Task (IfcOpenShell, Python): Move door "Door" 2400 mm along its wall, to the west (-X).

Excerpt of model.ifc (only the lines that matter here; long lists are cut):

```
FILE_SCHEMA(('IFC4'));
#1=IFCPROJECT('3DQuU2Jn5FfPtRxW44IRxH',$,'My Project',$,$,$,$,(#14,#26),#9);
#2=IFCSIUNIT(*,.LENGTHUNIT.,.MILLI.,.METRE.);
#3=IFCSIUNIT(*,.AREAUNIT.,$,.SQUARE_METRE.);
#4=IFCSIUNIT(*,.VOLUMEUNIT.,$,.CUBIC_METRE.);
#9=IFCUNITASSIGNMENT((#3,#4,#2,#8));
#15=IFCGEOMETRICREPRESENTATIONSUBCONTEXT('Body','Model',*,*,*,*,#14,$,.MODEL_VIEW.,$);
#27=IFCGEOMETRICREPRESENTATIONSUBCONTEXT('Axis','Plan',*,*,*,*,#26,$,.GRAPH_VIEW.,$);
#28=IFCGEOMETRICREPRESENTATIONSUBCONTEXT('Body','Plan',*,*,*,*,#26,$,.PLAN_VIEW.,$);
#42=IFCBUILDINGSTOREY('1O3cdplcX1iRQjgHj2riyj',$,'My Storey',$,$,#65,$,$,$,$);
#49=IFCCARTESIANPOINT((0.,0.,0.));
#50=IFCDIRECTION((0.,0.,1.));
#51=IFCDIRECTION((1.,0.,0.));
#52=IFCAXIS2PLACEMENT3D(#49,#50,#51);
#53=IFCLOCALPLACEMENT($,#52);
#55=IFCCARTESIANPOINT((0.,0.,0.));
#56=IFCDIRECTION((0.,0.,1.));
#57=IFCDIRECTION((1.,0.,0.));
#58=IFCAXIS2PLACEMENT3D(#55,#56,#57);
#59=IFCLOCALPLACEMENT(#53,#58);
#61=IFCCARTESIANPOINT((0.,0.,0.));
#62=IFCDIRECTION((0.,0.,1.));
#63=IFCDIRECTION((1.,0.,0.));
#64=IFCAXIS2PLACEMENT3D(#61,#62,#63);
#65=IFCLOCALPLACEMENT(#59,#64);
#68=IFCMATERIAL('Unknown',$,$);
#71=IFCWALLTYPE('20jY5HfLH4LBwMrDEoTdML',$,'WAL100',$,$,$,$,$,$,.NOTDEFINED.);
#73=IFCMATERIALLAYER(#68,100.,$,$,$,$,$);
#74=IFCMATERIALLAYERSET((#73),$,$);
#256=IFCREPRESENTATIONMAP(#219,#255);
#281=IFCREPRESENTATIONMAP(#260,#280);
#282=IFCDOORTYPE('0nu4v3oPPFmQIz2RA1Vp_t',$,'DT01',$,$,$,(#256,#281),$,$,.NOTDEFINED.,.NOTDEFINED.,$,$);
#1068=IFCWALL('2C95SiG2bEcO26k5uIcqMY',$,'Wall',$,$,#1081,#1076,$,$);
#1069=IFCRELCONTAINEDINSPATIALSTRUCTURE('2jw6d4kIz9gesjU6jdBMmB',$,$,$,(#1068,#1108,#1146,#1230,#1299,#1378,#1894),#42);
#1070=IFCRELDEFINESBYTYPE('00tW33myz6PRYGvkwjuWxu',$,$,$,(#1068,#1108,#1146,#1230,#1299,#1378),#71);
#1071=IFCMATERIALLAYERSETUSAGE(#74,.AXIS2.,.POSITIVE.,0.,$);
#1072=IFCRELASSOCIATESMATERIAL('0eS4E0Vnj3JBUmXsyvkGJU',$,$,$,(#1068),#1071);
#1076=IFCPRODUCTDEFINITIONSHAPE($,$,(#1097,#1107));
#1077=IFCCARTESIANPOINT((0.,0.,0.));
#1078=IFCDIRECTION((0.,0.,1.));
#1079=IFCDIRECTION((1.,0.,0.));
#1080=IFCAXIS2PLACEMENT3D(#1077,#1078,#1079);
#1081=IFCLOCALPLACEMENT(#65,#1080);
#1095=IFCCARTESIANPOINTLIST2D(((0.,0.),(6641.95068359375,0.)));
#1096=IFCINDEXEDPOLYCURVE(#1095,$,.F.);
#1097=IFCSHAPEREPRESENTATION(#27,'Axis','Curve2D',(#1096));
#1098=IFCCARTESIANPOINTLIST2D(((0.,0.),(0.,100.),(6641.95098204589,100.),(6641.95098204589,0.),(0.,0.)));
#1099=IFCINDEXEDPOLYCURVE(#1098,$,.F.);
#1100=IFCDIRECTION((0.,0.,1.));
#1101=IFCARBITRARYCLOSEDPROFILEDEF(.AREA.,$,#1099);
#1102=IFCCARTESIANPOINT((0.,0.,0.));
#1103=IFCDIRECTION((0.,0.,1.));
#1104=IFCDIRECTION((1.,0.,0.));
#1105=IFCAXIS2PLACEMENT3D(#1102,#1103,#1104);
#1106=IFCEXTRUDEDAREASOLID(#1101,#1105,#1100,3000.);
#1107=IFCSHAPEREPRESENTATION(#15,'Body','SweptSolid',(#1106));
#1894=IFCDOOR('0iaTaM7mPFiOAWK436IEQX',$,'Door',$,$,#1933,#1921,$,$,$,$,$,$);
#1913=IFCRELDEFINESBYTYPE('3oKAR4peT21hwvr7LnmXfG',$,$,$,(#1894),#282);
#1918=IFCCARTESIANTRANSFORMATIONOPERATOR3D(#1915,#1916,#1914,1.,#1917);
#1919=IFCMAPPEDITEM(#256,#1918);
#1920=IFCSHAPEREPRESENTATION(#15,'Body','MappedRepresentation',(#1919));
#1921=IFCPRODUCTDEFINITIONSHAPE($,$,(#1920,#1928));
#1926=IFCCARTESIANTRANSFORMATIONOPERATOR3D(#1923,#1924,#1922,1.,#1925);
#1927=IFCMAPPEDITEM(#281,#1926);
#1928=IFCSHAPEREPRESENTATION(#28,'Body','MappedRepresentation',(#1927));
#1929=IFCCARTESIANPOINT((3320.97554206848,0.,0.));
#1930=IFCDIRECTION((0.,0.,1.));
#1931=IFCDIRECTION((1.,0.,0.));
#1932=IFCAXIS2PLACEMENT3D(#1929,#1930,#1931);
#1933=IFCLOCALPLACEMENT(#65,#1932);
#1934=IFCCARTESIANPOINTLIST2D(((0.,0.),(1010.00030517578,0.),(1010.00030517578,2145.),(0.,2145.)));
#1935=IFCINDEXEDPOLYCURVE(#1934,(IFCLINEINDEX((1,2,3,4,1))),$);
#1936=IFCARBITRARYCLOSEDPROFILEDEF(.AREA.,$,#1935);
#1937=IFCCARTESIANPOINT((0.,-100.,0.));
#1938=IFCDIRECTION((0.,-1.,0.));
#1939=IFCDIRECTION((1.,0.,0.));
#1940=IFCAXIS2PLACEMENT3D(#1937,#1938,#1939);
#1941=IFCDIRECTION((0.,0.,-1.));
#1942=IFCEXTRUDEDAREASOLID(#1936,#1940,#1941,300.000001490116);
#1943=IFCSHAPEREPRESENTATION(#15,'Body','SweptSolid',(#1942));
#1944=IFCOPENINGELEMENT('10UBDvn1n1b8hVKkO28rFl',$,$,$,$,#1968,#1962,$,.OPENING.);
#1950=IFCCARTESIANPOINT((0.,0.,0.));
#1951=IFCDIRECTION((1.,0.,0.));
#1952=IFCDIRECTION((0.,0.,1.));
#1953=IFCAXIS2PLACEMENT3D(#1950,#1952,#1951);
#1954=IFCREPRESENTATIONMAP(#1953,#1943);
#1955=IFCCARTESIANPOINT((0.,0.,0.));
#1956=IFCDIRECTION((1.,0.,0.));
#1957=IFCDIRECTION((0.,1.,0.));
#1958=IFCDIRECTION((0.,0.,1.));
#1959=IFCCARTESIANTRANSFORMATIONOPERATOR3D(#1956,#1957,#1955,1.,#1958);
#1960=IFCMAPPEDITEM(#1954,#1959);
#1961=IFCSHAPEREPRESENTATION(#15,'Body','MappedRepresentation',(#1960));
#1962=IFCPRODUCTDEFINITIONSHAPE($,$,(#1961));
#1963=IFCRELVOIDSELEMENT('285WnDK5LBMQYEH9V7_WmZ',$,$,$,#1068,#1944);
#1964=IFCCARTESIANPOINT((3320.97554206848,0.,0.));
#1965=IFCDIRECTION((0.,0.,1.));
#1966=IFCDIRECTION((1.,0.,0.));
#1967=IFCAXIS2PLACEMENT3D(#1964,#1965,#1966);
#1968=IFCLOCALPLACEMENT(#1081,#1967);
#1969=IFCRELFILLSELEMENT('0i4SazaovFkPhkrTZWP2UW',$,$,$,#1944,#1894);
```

```python
import ifcopenshell
import ifcopenshell.api.geometry
import ifcopenshell.util.placement

model = ifcopenshell.open("model.ifc")

door = model.by_guid("0iaTaM7mPFiOAWK436IEQX")
opening = door.FillsVoids[0].RelatingOpeningElement
wall = opening.VoidsElements[0].RelatingBuildingElement

wall_matrix = ifcopenshell.util.placement.get_local_placement(wall.ObjectPlacement)
shift = wall_matrix[:3, 0] * -2400.0
before = ifcopenshell.util.placement.get_local_placement(door.ObjectPlacement)[:3, 3].copy()

# The door is not placed relative to its opening, so move both.
for product in (opening, door):
    matrix = ifcopenshell.util.placement.get_local_placement(product.ObjectPlacement)
    matrix[:3, 3] += shift
    ifcopenshell.api.geometry.edit_object_placement(model, product=product, matrix=matrix, is_si=False)

after = ifcopenshell.util.placement.get_local_placement(door.ObjectPlacement)[:3, 3]
print("door moved by", (after - before).round(3) + 0.0)

model.write("model-out.ifc")
```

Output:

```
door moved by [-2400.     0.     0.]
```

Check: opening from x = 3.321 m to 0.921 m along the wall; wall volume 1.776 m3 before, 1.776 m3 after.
